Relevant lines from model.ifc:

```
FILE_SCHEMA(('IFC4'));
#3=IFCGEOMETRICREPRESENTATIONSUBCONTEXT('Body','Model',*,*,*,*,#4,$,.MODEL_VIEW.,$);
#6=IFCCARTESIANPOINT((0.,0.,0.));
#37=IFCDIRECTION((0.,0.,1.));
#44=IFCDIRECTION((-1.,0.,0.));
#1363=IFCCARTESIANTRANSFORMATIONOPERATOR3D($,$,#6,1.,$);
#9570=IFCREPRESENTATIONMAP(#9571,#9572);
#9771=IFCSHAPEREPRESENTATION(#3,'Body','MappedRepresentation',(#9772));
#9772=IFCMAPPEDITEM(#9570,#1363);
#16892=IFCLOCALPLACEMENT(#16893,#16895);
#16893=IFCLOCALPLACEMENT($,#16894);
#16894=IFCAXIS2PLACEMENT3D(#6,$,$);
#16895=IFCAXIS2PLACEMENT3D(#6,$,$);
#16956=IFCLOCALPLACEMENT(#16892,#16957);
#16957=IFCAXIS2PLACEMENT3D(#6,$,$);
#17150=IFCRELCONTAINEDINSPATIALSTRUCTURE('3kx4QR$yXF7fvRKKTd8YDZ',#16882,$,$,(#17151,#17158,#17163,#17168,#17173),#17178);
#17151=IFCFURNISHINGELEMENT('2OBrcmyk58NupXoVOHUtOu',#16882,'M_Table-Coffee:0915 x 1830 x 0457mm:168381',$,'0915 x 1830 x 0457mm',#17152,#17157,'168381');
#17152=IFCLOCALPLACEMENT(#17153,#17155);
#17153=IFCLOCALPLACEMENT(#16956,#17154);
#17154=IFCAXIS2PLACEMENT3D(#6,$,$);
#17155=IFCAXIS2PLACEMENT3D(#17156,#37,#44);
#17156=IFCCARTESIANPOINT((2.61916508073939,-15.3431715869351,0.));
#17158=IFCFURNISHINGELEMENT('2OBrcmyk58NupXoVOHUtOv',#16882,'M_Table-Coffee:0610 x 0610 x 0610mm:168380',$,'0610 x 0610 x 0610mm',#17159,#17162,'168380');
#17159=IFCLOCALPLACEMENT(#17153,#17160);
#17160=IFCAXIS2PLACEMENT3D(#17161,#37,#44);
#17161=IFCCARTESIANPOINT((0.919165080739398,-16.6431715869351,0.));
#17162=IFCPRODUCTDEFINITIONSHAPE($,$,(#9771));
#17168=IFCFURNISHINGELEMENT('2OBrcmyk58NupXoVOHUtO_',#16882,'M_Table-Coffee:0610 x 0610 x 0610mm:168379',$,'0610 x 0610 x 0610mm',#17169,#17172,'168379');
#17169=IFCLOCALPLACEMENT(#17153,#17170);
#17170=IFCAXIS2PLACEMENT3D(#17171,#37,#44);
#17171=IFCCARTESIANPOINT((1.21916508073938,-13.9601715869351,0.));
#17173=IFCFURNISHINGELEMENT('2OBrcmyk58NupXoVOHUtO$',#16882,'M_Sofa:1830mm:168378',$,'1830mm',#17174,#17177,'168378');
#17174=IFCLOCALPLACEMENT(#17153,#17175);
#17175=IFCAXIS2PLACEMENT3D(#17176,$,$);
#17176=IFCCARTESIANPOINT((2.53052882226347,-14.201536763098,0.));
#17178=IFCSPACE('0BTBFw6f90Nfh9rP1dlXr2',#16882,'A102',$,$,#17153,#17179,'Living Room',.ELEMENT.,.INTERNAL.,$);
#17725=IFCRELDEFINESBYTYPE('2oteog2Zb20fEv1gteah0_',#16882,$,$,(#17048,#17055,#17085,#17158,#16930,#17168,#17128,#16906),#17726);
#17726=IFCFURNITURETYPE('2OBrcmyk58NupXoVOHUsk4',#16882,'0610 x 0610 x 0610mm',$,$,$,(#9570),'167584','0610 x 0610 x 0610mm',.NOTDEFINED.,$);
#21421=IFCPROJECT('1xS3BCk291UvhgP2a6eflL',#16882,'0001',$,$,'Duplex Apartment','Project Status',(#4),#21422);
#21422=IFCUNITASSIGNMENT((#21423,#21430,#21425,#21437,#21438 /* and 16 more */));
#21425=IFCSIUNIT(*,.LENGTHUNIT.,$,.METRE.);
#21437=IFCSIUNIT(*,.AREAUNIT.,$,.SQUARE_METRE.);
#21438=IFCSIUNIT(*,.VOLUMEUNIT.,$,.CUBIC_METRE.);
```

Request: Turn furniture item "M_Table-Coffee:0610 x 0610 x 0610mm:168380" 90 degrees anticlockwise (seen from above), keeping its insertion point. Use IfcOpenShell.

```python
import ifcopenshell
import ifcopenshell.api.geometry
import ifcopenshell.util.placement

model = ifcopenshell.open("model.ifc")

item = model.by_guid("2OBrcmyk58NupXoVOHUtOv")
matrix = ifcopenshell.util.placement.get_local_placement(item.ObjectPlacement)
matrix = matrix @ ifcopenshell.util.placement.rotation(90, "Z")
ifcopenshell.api.geometry.edit_object_placement(model, product=item, matrix=matrix, is_si=False)

print(ifcopenshell.util.placement.get_local_placement(item.ObjectPlacement).round(3) + 0.0)

model.write("model-out.ifc")
```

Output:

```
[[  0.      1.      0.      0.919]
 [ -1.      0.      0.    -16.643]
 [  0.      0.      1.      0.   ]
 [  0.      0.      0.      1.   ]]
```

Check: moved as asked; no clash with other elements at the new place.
